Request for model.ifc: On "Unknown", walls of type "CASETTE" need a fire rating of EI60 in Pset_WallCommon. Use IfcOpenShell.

First a look at what the model holds.

```python
import ifcopenshell
import ifcopenshell.util.element

model = ifcopenshell.open("model.ifc")
print(model.schema)
storey = next(s for s in model.by_type("IfcBuildingStorey") if s.Name == "Unknown")
walls = [e for e in ifcopenshell.util.element.get_decomposition(storey) if e.is_a("IfcWall")]
seen = {}
for e in walls:
    element_type = ifcopenshell.util.element.get_type(e)
    key = (element_type.Name if element_type != e and element_type else None, ifcopenshell.util.element.get_pset(e, "Pset_WallCommon", "FireRating"))
    seen[key] = seen.get(key, 0) + 1
for (name, value), count in sorted(seen.items(), key=str):
    print(count, "x", name, "|", value)
```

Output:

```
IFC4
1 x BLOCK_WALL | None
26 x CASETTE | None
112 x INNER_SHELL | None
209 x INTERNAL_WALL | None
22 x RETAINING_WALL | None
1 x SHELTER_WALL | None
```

```python
import ifcopenshell
import ifcopenshell.api.pset
import ifcopenshell.util.element

model = ifcopenshell.open("model.ifc")

storey = next(s for s in model.by_type("IfcBuildingStorey") if s.Name == "Unknown")
walls = [e for e in ifcopenshell.util.element.get_decomposition(storey) if e.is_a("IfcWall")]

count = 0
for e in walls:
    element_type = ifcopenshell.util.element.get_type(e)
    if element_type in (None, e) or element_type.Name != "CASETTE":
        continue
    found = ifcopenshell.util.element.get_pset(e, "Pset_WallCommon", should_inherit=False)
    if found:
        pset = model.by_id(found["id"])
        if len(ifcopenshell.util.element.get_elements_by_pset(pset)) > 1:
            pset = ifcopenshell.api.pset.unshare_pset(model, products=[e], pset=pset)[0]
    else:
        pset = ifcopenshell.api.pset.add_pset(model, product=e, name="Pset_WallCommon")
    ifcopenshell.api.pset.edit_pset(model, pset=pset, properties={"FireRating": "EI60"})
    count += 1

print(count, "walls updated")

model.write("model_updated.ifc")
```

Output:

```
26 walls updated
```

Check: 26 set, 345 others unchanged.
